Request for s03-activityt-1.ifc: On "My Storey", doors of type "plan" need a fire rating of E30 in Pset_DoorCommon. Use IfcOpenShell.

First a look at what the model holds.

```python
import ifcopenshell
import ifcopenshell.util.element

model = ifcopenshell.open("s03-activityt-1.ifc")
print(model.schema)
storey = next(s for s in model.by_type("IfcBuildingStorey") if s.Name == "My Storey")
doors = [e for e in ifcopenshell.util.element.get_decomposition(storey) if e.is_a("IfcDoor")]
seen = {}
for e in doors:
    element_type = ifcopenshell.util.element.get_type(e)
    key = (element_type.Name if element_type != e and element_type else None, ifcopenshell.util.element.get_pset(e, "Pset_DoorCommon", "FireRating"))
    seen[key] = seen.get(key, 0) + 1
for (name, value), count in sorted(seen.items(), key=str):
    print(count, "x", name, "|", value)
```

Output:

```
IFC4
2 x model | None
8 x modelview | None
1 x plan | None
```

```python
import ifcopenshell
import ifcopenshell.api.pset
import ifcopenshell.util.element

model = ifcopenshell.open("s03-activityt-1.ifc")

storey = next(s for s in model.by_type("IfcBuildingStorey") if s.Name == "My Storey")
doors = [e for e in ifcopenshell.util.element.get_decomposition(storey) if e.is_a("IfcDoor")]

count = 0
for e in doors:
    element_type = ifcopenshell.util.element.get_type(e)
    if element_type in (None, e) or element_type.Name != "plan":
        continue
    # add_pset returns the element's existing set when there is one.
    pset = ifcopenshell.api.pset.add_pset(model, product=e, name="Pset_DoorCommon")
    ifcopenshell.api.pset.edit_pset(model, pset=pset, properties={"FireRating": "E30"})
    count += 1

print(count, "doors updated")

model.write("s03-activityt-1-out.ifc")
```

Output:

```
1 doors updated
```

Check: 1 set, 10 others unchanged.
